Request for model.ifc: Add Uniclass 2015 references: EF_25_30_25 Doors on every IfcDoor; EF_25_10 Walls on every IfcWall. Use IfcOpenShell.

First a look at what the model holds.

```python
import ifcopenshell

model = ifcopenshell.open("model.ifc")
print(model.schema)
print("classifications:", [c.Name for c in model.by_type("IfcClassification")])
for ifc_class in ("IfcDoor", "IfcRoof", "IfcStair", "IfcWall", "IfcWindow"):
    print(ifc_class, len(model.by_type(ifc_class)))
```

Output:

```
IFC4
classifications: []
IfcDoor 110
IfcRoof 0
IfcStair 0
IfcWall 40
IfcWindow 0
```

```python
import ifcopenshell
import ifcopenshell.api.classification

model = ifcopenshell.open("model.ifc")

system = ifcopenshell.api.classification.add_classification(model, classification="Uniclass 2015")

codes = {
    "IfcDoor": ("EF_25_30_25", "Doors"),
    "IfcWall": ("EF_25_10", "Walls"),
}
for ifc_class, (code, name) in codes.items():
    products = model.by_type(ifc_class)
    ifcopenshell.api.classification.add_reference(
        model, products=products, classification=system, identification=code, name=name
    )
    print(code, len(products))

model.write("model-out.ifc")
```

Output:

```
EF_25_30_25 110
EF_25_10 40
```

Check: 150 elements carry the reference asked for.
